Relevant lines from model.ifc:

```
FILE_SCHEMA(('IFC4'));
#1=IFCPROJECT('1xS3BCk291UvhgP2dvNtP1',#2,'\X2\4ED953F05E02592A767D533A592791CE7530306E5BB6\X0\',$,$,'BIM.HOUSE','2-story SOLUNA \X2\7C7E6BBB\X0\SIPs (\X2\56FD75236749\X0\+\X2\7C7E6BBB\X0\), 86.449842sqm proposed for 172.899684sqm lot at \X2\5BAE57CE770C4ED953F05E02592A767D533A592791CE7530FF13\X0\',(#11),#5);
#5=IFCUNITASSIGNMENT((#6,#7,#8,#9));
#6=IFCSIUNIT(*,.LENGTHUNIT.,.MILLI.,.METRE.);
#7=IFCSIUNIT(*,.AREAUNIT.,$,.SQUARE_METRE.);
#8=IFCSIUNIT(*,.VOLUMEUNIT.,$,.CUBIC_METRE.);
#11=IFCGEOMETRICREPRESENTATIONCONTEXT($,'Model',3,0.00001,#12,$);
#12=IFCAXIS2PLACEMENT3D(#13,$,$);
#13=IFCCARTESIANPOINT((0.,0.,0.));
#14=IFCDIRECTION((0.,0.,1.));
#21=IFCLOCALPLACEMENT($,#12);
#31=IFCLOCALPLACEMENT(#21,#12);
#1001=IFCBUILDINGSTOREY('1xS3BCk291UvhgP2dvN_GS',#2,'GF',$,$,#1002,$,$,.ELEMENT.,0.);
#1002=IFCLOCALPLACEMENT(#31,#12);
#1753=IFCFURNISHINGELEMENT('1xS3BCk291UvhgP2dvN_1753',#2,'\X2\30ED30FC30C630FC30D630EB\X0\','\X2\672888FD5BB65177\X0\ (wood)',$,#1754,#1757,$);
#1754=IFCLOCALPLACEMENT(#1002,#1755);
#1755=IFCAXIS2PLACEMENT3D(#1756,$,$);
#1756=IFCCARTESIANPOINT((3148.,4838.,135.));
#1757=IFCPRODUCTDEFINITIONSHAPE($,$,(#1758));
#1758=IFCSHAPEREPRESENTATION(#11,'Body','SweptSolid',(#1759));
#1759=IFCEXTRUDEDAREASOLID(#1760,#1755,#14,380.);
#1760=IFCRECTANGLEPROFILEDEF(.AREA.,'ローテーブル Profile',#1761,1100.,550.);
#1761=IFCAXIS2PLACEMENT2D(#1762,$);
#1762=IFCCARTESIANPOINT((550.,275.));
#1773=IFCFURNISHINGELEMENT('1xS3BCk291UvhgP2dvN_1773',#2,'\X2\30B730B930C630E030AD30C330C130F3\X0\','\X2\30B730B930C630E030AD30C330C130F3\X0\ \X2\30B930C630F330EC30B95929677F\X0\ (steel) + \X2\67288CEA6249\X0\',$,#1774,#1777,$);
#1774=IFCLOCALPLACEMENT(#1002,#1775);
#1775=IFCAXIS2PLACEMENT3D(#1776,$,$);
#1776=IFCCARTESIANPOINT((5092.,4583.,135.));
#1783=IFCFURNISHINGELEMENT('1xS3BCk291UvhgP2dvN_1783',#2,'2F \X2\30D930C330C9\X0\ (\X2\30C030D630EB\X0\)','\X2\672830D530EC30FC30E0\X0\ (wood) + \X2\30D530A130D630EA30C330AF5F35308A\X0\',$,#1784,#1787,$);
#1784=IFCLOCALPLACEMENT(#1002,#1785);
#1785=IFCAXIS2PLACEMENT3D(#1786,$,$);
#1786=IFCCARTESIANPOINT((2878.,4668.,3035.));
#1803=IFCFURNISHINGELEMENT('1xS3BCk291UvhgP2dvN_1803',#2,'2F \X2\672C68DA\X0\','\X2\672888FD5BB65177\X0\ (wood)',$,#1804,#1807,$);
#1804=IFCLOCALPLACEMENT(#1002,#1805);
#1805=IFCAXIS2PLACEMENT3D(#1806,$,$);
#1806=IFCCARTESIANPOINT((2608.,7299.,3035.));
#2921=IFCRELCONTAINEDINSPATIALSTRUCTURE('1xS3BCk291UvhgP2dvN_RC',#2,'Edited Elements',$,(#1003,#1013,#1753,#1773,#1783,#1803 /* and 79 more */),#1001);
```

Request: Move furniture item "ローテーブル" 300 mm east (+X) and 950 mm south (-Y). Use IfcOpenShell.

```python
import ifcopenshell
import ifcopenshell.api.geometry
import ifcopenshell.util.placement

model = ifcopenshell.open("model.ifc")

item = model.by_guid("1xS3BCk291UvhgP2dvN_1753")
matrix = ifcopenshell.util.placement.get_local_placement(item.ObjectPlacement)
matrix[0, 3] += 300.0
matrix[1, 3] -= 950.0
ifcopenshell.api.geometry.edit_object_placement(model, product=item, matrix=matrix, is_si=False)

print(ifcopenshell.util.placement.get_local_placement(item.ObjectPlacement).round(3) + 0.0)

model.write("model-out.ifc")
```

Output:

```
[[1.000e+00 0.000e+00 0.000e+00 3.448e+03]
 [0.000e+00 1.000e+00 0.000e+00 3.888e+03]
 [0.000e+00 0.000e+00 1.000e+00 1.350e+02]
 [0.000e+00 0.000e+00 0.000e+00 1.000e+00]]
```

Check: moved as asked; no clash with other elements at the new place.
